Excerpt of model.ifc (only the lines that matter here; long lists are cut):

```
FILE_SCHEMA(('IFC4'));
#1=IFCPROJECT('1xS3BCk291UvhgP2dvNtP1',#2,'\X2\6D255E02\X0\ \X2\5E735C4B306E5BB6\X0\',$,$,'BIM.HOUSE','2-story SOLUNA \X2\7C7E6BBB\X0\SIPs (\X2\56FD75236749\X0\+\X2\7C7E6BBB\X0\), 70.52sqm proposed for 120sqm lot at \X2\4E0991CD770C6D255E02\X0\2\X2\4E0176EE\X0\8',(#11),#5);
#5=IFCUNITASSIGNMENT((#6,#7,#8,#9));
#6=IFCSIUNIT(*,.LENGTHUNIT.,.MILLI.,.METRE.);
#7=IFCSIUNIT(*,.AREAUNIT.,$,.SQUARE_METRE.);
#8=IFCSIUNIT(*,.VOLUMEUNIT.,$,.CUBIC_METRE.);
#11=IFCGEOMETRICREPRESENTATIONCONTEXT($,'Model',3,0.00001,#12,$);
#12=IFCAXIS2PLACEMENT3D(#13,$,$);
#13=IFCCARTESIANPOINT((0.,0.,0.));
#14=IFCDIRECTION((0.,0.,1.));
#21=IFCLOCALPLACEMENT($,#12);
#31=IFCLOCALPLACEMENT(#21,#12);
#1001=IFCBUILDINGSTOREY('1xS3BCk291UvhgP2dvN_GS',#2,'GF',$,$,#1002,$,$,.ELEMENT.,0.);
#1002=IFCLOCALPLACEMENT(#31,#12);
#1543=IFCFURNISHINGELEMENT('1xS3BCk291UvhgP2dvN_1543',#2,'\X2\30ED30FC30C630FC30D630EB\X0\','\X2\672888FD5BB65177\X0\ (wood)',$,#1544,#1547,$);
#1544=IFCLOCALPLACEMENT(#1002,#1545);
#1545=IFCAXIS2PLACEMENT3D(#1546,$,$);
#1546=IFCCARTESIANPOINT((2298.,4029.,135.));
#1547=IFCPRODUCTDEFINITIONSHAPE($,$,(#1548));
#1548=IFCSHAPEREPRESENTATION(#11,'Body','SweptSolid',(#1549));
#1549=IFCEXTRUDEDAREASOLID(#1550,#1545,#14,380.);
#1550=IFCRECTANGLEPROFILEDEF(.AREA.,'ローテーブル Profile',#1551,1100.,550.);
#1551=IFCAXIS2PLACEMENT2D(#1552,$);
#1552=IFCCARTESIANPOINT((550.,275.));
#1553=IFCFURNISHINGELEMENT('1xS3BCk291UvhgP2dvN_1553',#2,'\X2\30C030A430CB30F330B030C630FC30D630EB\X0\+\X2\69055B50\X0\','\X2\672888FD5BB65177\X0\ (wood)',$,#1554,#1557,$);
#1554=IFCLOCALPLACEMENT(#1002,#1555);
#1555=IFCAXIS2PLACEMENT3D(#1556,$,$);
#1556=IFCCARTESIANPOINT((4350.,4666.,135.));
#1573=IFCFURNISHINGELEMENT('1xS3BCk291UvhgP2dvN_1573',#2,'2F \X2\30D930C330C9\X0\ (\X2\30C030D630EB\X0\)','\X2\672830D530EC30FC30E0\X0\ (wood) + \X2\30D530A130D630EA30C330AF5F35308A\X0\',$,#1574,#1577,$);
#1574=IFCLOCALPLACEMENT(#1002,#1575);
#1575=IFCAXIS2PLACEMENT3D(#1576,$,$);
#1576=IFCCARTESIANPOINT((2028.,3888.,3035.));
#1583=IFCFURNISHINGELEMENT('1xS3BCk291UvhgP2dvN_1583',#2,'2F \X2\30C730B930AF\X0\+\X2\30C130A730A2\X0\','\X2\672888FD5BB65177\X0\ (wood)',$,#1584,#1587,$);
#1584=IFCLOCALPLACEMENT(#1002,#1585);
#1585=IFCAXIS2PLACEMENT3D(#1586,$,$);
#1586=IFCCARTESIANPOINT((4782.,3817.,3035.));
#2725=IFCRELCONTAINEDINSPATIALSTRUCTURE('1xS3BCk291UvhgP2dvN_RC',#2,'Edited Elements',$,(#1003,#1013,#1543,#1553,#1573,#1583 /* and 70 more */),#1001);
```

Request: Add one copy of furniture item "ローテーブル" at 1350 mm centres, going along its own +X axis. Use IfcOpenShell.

```python
import ifcopenshell
import ifcopenshell.api.geometry
import ifcopenshell.api.root
import ifcopenshell.util.element
import ifcopenshell.util.placement
import ifcopenshell.util.unit

model = ifcopenshell.open("model.ifc")
unit_scale = ifcopenshell.util.unit.calculate_unit_scale(model)


def reuse_history(source, copy):
    """copy_class also copies each property set's owner history, people and application; keep the originals."""
    for rel in copy.IsDefinedBy:
        if rel.is_a("IfcRelDefinesByProperties") and (history := rel.RelatingPropertyDefinition.OwnerHistory):
            rel.RelatingPropertyDefinition.OwnerHistory = source.OwnerHistory
            ifcopenshell.util.element.remove_deep2(model, history)


source = model.by_id(1543)
base = ifcopenshell.util.placement.get_local_placement(source.ObjectPlacement)
step = base[:3, 0] * 1.35 / unit_scale

for i in range(1, 2):
    copy = ifcopenshell.api.root.copy_class(model, product=source)
    copy.Representation = ifcopenshell.util.element.copy_deep(
        model, source.Representation, exclude=["IfcGeometricRepresentationContext", "IfcRepresentationMap"]
    )
    reuse_history(source, copy)
    matrix = base.copy()
    matrix[:3, 3] += i * step
    print("added at", matrix[:3, 3].round(3) + 0.0)
    ifcopenshell.api.geometry.edit_object_placement(model, product=copy, matrix=matrix, is_si=False)

model.write("model_rev.ifc")
```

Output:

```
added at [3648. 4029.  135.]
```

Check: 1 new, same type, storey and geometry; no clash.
